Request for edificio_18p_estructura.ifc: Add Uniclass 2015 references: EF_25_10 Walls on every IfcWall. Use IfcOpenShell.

First a look at what the model holds.

```python
import ifcopenshell

model = ifcopenshell.open("edificio_18p_estructura.ifc")
print(model.schema)
print("classifications:", [c.Name for c in model.by_type("IfcClassification")])
for ifc_class in ("IfcDoor", "IfcRoof", "IfcStair", "IfcWall", "IfcWindow"):
    print(ifc_class, len(model.by_type(ifc_class)))
```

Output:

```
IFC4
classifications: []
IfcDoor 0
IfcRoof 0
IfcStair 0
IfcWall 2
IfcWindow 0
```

```python
import ifcopenshell
import ifcopenshell.api.classification

model = ifcopenshell.open("edificio_18p_estructura.ifc")

system = ifcopenshell.api.classification.add_classification(model, classification="Uniclass 2015")

codes = {
    "IfcWall": ("EF_25_10", "Walls"),
}
for ifc_class, (code, name) in codes.items():
    products = model.by_type(ifc_class)
    ifcopenshell.api.classification.add_reference(
        model, products=products, classification=system, identification=code, name=name
    )
    print(code, len(products))

model.write("edificio_18p_estructura_v2.ifc")
```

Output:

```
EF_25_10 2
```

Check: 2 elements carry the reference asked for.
